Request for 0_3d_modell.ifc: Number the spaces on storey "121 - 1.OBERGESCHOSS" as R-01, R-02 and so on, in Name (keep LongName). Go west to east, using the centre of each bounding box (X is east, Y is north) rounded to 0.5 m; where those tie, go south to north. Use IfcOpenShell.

First a look at what the model holds.

```python
import ifcopenshell
import ifcopenshell.util.element
import ifcopenshell.util.placement

model = ifcopenshell.open("0_3d_modell.ifc")
print(model.schema)
storey = next(s for s in model.by_type("IfcBuildingStorey") if s.Name == "121 - 1.OBERGESCHOSS")
spaces = [e for e in ifcopenshell.util.element.get_decomposition(storey) if e.is_a("IfcSpace")]
for e in sorted(spaces, key=lambda e: e.id()):
    origin = ifcopenshell.util.placement.get_local_placement(e.ObjectPlacement)[:3, 3]
    print(e.id(), e.Name, e.LongName, origin.round(2) + 0.0, sep=" | ")
```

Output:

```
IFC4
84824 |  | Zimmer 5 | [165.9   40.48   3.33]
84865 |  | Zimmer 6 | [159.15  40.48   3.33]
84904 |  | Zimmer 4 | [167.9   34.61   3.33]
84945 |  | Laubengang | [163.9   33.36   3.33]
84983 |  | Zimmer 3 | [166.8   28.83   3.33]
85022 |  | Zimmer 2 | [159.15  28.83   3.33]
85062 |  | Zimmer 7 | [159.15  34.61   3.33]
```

```python
import ifcopenshell
import ifcopenshell.geom
import ifcopenshell.util.element
import ifcopenshell.util.shape

model = ifcopenshell.open("0_3d_modell.ifc")
settings = ifcopenshell.geom.settings()
settings.set("use-world-coords", True)


def centre(element):
    shape = ifcopenshell.geom.create_shape(settings, element)
    return ifcopenshell.util.shape.get_bbox_centroid(shape.geometry)


storey = next(s for s in model.by_type("IfcBuildingStorey") if s.Name == "121 - 1.OBERGESCHOSS")
spaces = [e for e in ifcopenshell.util.element.get_decomposition(storey) if e.is_a("IfcSpace")]

# Insertion points can sit at a corner or the storey origin, so sort by the geometry (in metres).
centres = {e: centre(e) for e in spaces}
spaces.sort(key=lambda e: (round(centres[e][0] / 0.5), centres[e][1]))

for i, e in enumerate(spaces, start=1):
    number = f"R-{i:02d}"
    e.Name = number
    print(e.id(), number)

model.write("0_3d_modell-out.ifc")
```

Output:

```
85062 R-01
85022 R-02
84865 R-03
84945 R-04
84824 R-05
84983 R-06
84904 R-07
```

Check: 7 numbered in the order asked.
